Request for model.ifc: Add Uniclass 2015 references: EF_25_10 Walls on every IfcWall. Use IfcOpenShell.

First a look at what the model holds.

```python
import ifcopenshell

model = ifcopenshell.open("model.ifc")
print(model.schema)
print("classifications:", [c.Name for c in model.by_type("IfcClassification")])
for ifc_class in ("IfcDoor", "IfcRoof", "IfcStair", "IfcWall", "IfcWindow"):
    print(ifc_class, len(model.by_type(ifc_class)))
```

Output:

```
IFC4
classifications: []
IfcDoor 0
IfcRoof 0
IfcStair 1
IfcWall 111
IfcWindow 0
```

```python
import ifcopenshell
import ifcopenshell.api.classification

model = ifcopenshell.open("model.ifc")

system = ifcopenshell.api.classification.add_classification(model, classification="Uniclass 2015")

codes = {
    "IfcWall": ("EF_25_10", "Walls"),
}
for ifc_class, (code, name) in codes.items():
    products = model.by_type(ifc_class)
    ifcopenshell.api.classification.add_reference(
        model, products=products, classification=system, identification=code, name=name
    )
    print(code, len(products))

model.write("model_rev.ifc")
```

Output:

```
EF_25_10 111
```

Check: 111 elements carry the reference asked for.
